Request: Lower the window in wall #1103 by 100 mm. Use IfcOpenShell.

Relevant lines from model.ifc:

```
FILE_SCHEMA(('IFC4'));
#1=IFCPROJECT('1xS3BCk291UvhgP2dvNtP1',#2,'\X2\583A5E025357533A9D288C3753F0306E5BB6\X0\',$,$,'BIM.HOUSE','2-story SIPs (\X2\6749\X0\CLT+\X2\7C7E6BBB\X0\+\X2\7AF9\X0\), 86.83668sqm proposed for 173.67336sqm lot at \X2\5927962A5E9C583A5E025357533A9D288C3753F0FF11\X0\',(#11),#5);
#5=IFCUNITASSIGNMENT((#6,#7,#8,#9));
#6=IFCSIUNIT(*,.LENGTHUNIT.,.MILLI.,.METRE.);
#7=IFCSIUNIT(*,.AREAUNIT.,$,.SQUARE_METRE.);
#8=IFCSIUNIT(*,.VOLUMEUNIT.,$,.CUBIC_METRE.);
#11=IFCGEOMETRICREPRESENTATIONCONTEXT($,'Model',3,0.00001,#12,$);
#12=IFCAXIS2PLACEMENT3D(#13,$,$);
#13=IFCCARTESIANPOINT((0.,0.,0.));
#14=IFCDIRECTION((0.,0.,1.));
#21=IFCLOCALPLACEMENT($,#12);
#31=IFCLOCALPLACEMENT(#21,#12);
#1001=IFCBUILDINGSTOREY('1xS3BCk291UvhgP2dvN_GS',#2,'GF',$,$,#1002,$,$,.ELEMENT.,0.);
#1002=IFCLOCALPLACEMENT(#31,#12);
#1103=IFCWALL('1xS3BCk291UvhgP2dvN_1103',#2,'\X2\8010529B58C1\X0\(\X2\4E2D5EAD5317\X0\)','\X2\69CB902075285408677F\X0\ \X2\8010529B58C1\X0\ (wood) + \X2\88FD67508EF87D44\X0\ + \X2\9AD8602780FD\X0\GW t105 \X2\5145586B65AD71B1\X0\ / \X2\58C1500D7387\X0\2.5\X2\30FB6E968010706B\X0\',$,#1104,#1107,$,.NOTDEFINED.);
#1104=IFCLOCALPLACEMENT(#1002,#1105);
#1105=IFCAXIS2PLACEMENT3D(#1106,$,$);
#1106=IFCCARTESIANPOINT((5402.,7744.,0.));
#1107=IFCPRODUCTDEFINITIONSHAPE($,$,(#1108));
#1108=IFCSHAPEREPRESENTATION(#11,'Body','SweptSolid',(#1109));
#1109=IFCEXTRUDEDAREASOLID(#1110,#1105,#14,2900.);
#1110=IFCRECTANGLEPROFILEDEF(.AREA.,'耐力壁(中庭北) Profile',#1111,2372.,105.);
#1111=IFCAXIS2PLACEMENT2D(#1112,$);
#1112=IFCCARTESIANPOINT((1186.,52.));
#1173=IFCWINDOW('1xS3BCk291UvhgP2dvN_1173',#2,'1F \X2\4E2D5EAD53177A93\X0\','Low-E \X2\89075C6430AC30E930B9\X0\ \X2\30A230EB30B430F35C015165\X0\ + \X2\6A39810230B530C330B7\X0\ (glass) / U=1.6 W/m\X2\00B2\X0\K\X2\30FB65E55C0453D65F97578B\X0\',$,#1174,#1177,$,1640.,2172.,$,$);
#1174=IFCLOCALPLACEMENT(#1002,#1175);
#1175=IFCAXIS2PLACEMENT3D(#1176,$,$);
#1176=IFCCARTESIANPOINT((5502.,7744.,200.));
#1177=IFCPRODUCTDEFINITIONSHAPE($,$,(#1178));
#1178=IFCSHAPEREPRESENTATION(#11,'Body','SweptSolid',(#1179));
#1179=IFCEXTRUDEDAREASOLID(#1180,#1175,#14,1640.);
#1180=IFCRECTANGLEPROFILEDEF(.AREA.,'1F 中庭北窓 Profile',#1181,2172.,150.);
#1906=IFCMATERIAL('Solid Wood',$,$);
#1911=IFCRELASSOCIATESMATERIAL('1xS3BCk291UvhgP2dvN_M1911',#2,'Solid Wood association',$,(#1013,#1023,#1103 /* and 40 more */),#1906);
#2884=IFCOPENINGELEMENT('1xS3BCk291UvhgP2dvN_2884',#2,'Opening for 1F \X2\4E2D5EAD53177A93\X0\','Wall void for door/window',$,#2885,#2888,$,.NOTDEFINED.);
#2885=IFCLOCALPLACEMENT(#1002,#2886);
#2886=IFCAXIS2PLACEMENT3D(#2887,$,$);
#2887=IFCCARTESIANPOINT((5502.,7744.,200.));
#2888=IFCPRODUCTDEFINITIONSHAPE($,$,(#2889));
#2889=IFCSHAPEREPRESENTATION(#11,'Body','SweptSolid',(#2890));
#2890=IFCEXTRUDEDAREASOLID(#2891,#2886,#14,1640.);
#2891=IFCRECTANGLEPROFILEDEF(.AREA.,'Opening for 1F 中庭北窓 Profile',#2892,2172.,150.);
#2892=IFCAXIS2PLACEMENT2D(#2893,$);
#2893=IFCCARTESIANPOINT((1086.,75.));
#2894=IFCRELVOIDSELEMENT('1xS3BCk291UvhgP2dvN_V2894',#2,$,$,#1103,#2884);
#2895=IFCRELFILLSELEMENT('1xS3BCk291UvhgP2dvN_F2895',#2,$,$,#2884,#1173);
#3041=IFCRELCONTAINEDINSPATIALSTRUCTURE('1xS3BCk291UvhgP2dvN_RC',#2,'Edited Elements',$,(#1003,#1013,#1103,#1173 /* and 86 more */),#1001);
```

```python
import numpy as np
import ifcopenshell
import ifcopenshell.api.geometry
import ifcopenshell.util.placement
import ifcopenshell.util.unit

model = ifcopenshell.open("model.ifc")
unit_scale = ifcopenshell.util.unit.calculate_unit_scale(model)

window = model.by_guid("1xS3BCk291UvhgP2dvN_1173")
opening = window.FillsVoids[0].RelatingOpeningElement
dz = -100.0

shift = np.array([0.0, 0.0, dz])
# The window is not placed relative to its opening, so move both.
for product in (opening, window):
    matrix = ifcopenshell.util.placement.get_local_placement(product.ObjectPlacement)
    matrix[:3, 3] += shift
    ifcopenshell.api.geometry.edit_object_placement(model, product=product, matrix=matrix, is_si=False)

print(f"moved by {dz * unit_scale:+.3f} m")

model.write("model_v2.ifc")
```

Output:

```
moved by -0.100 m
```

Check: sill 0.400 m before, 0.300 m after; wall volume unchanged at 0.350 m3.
